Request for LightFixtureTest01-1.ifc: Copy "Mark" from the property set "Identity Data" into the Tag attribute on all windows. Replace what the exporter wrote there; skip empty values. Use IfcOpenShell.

First a look at what the model holds.

```python
import ifcopenshell
import ifcopenshell.util.element

model = ifcopenshell.open("LightFixtureTest01-1.ifc")
print(model.schema)
windows = model.by_type("IfcWindow")
print(len(windows), "windows")
for e in windows[:8]:
    source = ifcopenshell.util.element.get_pset(e, "Identity Data", "Mark")
    target = e.Tag
    print(e.id(), repr(source), repr(target), sep=" | ")
```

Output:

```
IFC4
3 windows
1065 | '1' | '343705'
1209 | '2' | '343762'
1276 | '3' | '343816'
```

```python
import ifcopenshell
import ifcopenshell.util.element

model = ifcopenshell.open("LightFixtureTest01-1.ifc")

count = 0
for e in model.by_type("IfcWindow"):
    value = ifcopenshell.util.element.get_pset(e, "Identity Data", "Mark")
    current = e.Tag
    if not value or not value.strip() or current == value:
        continue
    e.Tag = value
    count += 1

print(count, "windows updated")

model.write("LightFixtureTest01-1_v2.ifc")
```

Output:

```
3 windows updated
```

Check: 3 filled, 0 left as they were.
